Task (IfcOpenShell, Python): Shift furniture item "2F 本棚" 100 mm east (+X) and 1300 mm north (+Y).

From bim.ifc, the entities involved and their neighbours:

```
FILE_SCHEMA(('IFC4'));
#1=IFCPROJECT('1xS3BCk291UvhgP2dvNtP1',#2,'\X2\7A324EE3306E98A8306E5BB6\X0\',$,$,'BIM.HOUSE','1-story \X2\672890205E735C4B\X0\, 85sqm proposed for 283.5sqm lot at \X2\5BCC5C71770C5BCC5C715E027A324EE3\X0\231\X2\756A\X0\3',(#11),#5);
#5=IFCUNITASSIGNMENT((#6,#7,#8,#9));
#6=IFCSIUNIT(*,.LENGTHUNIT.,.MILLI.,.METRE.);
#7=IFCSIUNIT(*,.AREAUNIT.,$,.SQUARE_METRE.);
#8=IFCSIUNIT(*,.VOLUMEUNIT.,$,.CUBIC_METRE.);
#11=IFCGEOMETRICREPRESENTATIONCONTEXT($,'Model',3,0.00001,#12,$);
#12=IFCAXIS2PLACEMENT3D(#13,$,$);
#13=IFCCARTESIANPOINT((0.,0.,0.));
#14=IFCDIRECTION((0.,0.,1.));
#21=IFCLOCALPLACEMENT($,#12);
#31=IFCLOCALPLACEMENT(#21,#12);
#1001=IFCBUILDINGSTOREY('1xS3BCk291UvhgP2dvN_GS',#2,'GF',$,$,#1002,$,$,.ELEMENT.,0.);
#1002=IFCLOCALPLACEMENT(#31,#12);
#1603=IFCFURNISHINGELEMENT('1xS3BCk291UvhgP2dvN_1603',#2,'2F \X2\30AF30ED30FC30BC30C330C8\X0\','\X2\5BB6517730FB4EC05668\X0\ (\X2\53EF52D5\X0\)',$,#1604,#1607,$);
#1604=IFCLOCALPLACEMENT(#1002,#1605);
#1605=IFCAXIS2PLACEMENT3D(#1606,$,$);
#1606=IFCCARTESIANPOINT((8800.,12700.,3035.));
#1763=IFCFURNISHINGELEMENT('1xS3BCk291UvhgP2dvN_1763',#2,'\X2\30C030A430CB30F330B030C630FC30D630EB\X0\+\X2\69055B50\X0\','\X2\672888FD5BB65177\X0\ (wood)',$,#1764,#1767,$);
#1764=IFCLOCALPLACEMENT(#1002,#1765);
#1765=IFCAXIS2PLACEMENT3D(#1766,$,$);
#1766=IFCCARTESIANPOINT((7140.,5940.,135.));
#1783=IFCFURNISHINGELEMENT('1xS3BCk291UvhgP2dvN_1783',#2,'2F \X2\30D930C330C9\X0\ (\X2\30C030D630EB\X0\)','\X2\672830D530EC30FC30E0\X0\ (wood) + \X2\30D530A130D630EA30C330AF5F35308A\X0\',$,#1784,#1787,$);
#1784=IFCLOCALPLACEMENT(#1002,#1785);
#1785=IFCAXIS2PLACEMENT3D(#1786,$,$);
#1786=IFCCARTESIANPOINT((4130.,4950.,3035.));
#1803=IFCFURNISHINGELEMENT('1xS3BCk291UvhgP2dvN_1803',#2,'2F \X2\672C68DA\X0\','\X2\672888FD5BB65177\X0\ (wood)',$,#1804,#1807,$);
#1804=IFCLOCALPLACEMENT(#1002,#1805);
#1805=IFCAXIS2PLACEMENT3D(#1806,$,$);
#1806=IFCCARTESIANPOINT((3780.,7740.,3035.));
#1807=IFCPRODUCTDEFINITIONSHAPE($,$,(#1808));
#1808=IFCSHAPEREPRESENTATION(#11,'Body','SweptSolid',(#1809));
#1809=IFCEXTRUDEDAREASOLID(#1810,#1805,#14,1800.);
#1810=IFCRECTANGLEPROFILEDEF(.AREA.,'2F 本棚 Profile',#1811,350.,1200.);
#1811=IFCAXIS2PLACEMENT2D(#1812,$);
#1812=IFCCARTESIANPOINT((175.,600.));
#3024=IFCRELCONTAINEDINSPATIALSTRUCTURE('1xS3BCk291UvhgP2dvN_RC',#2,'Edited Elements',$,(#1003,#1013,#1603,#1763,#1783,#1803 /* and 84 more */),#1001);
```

```python
import ifcopenshell
import ifcopenshell.api.geometry
import ifcopenshell.util.placement

model = ifcopenshell.open("bim.ifc")

item = model.by_id(1803)
matrix = ifcopenshell.util.placement.get_local_placement(item.ObjectPlacement)
matrix[0, 3] += 100.0
matrix[1, 3] += 1300.0
ifcopenshell.api.geometry.edit_object_placement(model, product=item, matrix=matrix, is_si=False)

print(ifcopenshell.util.placement.get_local_placement(item.ObjectPlacement).round(3) + 0.0)

model.write("bim_v2.ifc")
```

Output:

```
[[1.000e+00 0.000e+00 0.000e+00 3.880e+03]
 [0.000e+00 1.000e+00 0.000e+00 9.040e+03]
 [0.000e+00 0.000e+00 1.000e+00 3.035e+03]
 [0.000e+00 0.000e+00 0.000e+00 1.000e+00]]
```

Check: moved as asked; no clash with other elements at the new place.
